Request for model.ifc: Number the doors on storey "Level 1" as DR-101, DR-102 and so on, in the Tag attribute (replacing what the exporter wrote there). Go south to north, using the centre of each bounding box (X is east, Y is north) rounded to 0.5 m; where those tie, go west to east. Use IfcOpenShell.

First a look at what the model holds.

```python
import ifcopenshell
import ifcopenshell.util.element
import ifcopenshell.util.placement

model = ifcopenshell.open("model.ifc")
print(model.schema)
storey = next(s for s in model.by_type("IfcBuildingStorey") if s.Name == "Level 1")
doors = [e for e in ifcopenshell.util.element.get_decomposition(storey) if e.is_a("IfcDoor")]
for e in sorted(doors, key=lambda e: e.id()):
    origin = ifcopenshell.util.placement.get_local_placement(e.ObjectPlacement)[:3, 3]
    print(e.id(), e.Tag, e.Name, origin.round(2) + 0.0, sep=" | ")
```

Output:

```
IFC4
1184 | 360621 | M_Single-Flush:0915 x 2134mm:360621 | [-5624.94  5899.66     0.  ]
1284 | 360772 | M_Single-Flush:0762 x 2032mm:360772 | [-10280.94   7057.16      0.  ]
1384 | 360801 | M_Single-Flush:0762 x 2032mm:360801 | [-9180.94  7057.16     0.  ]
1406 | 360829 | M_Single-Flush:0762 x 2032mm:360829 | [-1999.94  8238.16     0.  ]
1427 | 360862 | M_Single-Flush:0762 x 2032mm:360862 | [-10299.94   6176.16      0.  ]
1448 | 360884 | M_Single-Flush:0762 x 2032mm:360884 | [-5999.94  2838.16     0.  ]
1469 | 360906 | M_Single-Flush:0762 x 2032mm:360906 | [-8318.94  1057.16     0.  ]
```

```python
import ifcopenshell
import ifcopenshell.geom
import ifcopenshell.util.element
import ifcopenshell.util.shape

model = ifcopenshell.open("model.ifc")
settings = ifcopenshell.geom.settings()
settings.set("use-world-coords", True)


def centre(element):
    shape = ifcopenshell.geom.create_shape(settings, element)
    return ifcopenshell.util.shape.get_bbox_centroid(shape.geometry)


storey = next(s for s in model.by_type("IfcBuildingStorey") if s.Name == "Level 1")
doors = [e for e in ifcopenshell.util.element.get_decomposition(storey) if e.is_a("IfcDoor")]

# Insertion points can sit at a corner or the storey origin, so sort by the geometry (in metres).
centres = {e: centre(e) for e in doors}
doors.sort(key=lambda e: (round(centres[e][1] / 0.5), centres[e][0]))

for i, e in enumerate(doors, start=1):
    number = f"DR-1{i:02d}"
    e.Tag = number
    print(e.id(), number)

model.write("model_edited.ifc")
```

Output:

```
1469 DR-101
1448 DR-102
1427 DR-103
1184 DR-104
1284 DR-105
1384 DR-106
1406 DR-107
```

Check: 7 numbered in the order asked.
